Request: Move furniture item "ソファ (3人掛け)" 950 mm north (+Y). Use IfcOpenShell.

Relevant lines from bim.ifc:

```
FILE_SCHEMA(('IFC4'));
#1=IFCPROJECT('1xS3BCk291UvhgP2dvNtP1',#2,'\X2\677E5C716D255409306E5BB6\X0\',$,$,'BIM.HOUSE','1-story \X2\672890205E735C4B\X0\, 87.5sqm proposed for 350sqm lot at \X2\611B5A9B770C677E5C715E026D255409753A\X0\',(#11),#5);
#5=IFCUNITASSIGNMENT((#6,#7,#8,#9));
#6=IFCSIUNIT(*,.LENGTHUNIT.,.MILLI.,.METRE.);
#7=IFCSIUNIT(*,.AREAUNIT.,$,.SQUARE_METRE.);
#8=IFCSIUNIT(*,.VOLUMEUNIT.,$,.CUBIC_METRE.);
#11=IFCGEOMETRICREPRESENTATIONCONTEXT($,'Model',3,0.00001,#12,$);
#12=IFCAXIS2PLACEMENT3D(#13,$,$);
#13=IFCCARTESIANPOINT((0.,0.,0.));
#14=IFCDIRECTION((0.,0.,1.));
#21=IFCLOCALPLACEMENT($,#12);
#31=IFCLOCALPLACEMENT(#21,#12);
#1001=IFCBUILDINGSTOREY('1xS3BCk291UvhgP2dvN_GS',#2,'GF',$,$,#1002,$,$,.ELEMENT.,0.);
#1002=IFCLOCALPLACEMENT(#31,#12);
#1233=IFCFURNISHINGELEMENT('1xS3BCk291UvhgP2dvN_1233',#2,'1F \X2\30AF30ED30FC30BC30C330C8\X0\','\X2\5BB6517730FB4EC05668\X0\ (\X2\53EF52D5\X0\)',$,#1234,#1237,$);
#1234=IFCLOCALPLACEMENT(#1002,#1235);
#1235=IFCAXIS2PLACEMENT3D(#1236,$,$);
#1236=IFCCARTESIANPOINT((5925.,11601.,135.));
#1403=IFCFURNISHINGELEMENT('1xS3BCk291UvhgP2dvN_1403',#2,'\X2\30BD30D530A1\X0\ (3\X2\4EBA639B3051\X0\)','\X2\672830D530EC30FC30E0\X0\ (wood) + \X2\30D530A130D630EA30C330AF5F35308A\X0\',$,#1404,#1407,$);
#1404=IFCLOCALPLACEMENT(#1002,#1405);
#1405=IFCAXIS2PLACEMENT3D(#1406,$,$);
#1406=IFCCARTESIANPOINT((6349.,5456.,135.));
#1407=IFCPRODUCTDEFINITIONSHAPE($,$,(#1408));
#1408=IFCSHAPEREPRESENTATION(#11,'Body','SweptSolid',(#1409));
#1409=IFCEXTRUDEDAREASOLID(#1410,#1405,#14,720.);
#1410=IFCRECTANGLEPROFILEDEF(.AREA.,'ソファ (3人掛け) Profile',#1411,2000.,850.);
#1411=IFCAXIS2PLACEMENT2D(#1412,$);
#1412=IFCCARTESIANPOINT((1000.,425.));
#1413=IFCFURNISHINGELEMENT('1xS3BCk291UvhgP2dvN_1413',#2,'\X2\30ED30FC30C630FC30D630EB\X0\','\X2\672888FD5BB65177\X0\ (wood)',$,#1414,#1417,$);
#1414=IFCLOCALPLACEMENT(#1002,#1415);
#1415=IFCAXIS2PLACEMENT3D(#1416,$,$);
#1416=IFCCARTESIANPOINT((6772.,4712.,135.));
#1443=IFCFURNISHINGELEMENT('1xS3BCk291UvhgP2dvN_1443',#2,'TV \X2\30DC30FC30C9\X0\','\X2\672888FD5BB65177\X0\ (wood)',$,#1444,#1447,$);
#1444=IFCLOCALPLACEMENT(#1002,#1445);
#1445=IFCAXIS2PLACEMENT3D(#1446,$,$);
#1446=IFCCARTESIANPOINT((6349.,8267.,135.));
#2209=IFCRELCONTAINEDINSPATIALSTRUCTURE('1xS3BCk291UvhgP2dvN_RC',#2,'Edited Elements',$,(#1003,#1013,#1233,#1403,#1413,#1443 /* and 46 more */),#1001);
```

```python
import ifcopenshell
import ifcopenshell.api.geometry
import ifcopenshell.util.placement
import ifcopenshell.util.unit

model = ifcopenshell.open("bim.ifc")
unit_scale = ifcopenshell.util.unit.calculate_unit_scale(model)

item = model.by_guid("1xS3BCk291UvhgP2dvN_1403")
matrix = ifcopenshell.util.placement.get_local_placement(item.ObjectPlacement)
matrix[1, 3] += 0.95 / unit_scale
ifcopenshell.api.geometry.edit_object_placement(model, product=item, matrix=matrix, is_si=False)

print(ifcopenshell.util.placement.get_local_placement(item.ObjectPlacement).round(3) + 0.0)

model.write("bim_updated.ifc")
```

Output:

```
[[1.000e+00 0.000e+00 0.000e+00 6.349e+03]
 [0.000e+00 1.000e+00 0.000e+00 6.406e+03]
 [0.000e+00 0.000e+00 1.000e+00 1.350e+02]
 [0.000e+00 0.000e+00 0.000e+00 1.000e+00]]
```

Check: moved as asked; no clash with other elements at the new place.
